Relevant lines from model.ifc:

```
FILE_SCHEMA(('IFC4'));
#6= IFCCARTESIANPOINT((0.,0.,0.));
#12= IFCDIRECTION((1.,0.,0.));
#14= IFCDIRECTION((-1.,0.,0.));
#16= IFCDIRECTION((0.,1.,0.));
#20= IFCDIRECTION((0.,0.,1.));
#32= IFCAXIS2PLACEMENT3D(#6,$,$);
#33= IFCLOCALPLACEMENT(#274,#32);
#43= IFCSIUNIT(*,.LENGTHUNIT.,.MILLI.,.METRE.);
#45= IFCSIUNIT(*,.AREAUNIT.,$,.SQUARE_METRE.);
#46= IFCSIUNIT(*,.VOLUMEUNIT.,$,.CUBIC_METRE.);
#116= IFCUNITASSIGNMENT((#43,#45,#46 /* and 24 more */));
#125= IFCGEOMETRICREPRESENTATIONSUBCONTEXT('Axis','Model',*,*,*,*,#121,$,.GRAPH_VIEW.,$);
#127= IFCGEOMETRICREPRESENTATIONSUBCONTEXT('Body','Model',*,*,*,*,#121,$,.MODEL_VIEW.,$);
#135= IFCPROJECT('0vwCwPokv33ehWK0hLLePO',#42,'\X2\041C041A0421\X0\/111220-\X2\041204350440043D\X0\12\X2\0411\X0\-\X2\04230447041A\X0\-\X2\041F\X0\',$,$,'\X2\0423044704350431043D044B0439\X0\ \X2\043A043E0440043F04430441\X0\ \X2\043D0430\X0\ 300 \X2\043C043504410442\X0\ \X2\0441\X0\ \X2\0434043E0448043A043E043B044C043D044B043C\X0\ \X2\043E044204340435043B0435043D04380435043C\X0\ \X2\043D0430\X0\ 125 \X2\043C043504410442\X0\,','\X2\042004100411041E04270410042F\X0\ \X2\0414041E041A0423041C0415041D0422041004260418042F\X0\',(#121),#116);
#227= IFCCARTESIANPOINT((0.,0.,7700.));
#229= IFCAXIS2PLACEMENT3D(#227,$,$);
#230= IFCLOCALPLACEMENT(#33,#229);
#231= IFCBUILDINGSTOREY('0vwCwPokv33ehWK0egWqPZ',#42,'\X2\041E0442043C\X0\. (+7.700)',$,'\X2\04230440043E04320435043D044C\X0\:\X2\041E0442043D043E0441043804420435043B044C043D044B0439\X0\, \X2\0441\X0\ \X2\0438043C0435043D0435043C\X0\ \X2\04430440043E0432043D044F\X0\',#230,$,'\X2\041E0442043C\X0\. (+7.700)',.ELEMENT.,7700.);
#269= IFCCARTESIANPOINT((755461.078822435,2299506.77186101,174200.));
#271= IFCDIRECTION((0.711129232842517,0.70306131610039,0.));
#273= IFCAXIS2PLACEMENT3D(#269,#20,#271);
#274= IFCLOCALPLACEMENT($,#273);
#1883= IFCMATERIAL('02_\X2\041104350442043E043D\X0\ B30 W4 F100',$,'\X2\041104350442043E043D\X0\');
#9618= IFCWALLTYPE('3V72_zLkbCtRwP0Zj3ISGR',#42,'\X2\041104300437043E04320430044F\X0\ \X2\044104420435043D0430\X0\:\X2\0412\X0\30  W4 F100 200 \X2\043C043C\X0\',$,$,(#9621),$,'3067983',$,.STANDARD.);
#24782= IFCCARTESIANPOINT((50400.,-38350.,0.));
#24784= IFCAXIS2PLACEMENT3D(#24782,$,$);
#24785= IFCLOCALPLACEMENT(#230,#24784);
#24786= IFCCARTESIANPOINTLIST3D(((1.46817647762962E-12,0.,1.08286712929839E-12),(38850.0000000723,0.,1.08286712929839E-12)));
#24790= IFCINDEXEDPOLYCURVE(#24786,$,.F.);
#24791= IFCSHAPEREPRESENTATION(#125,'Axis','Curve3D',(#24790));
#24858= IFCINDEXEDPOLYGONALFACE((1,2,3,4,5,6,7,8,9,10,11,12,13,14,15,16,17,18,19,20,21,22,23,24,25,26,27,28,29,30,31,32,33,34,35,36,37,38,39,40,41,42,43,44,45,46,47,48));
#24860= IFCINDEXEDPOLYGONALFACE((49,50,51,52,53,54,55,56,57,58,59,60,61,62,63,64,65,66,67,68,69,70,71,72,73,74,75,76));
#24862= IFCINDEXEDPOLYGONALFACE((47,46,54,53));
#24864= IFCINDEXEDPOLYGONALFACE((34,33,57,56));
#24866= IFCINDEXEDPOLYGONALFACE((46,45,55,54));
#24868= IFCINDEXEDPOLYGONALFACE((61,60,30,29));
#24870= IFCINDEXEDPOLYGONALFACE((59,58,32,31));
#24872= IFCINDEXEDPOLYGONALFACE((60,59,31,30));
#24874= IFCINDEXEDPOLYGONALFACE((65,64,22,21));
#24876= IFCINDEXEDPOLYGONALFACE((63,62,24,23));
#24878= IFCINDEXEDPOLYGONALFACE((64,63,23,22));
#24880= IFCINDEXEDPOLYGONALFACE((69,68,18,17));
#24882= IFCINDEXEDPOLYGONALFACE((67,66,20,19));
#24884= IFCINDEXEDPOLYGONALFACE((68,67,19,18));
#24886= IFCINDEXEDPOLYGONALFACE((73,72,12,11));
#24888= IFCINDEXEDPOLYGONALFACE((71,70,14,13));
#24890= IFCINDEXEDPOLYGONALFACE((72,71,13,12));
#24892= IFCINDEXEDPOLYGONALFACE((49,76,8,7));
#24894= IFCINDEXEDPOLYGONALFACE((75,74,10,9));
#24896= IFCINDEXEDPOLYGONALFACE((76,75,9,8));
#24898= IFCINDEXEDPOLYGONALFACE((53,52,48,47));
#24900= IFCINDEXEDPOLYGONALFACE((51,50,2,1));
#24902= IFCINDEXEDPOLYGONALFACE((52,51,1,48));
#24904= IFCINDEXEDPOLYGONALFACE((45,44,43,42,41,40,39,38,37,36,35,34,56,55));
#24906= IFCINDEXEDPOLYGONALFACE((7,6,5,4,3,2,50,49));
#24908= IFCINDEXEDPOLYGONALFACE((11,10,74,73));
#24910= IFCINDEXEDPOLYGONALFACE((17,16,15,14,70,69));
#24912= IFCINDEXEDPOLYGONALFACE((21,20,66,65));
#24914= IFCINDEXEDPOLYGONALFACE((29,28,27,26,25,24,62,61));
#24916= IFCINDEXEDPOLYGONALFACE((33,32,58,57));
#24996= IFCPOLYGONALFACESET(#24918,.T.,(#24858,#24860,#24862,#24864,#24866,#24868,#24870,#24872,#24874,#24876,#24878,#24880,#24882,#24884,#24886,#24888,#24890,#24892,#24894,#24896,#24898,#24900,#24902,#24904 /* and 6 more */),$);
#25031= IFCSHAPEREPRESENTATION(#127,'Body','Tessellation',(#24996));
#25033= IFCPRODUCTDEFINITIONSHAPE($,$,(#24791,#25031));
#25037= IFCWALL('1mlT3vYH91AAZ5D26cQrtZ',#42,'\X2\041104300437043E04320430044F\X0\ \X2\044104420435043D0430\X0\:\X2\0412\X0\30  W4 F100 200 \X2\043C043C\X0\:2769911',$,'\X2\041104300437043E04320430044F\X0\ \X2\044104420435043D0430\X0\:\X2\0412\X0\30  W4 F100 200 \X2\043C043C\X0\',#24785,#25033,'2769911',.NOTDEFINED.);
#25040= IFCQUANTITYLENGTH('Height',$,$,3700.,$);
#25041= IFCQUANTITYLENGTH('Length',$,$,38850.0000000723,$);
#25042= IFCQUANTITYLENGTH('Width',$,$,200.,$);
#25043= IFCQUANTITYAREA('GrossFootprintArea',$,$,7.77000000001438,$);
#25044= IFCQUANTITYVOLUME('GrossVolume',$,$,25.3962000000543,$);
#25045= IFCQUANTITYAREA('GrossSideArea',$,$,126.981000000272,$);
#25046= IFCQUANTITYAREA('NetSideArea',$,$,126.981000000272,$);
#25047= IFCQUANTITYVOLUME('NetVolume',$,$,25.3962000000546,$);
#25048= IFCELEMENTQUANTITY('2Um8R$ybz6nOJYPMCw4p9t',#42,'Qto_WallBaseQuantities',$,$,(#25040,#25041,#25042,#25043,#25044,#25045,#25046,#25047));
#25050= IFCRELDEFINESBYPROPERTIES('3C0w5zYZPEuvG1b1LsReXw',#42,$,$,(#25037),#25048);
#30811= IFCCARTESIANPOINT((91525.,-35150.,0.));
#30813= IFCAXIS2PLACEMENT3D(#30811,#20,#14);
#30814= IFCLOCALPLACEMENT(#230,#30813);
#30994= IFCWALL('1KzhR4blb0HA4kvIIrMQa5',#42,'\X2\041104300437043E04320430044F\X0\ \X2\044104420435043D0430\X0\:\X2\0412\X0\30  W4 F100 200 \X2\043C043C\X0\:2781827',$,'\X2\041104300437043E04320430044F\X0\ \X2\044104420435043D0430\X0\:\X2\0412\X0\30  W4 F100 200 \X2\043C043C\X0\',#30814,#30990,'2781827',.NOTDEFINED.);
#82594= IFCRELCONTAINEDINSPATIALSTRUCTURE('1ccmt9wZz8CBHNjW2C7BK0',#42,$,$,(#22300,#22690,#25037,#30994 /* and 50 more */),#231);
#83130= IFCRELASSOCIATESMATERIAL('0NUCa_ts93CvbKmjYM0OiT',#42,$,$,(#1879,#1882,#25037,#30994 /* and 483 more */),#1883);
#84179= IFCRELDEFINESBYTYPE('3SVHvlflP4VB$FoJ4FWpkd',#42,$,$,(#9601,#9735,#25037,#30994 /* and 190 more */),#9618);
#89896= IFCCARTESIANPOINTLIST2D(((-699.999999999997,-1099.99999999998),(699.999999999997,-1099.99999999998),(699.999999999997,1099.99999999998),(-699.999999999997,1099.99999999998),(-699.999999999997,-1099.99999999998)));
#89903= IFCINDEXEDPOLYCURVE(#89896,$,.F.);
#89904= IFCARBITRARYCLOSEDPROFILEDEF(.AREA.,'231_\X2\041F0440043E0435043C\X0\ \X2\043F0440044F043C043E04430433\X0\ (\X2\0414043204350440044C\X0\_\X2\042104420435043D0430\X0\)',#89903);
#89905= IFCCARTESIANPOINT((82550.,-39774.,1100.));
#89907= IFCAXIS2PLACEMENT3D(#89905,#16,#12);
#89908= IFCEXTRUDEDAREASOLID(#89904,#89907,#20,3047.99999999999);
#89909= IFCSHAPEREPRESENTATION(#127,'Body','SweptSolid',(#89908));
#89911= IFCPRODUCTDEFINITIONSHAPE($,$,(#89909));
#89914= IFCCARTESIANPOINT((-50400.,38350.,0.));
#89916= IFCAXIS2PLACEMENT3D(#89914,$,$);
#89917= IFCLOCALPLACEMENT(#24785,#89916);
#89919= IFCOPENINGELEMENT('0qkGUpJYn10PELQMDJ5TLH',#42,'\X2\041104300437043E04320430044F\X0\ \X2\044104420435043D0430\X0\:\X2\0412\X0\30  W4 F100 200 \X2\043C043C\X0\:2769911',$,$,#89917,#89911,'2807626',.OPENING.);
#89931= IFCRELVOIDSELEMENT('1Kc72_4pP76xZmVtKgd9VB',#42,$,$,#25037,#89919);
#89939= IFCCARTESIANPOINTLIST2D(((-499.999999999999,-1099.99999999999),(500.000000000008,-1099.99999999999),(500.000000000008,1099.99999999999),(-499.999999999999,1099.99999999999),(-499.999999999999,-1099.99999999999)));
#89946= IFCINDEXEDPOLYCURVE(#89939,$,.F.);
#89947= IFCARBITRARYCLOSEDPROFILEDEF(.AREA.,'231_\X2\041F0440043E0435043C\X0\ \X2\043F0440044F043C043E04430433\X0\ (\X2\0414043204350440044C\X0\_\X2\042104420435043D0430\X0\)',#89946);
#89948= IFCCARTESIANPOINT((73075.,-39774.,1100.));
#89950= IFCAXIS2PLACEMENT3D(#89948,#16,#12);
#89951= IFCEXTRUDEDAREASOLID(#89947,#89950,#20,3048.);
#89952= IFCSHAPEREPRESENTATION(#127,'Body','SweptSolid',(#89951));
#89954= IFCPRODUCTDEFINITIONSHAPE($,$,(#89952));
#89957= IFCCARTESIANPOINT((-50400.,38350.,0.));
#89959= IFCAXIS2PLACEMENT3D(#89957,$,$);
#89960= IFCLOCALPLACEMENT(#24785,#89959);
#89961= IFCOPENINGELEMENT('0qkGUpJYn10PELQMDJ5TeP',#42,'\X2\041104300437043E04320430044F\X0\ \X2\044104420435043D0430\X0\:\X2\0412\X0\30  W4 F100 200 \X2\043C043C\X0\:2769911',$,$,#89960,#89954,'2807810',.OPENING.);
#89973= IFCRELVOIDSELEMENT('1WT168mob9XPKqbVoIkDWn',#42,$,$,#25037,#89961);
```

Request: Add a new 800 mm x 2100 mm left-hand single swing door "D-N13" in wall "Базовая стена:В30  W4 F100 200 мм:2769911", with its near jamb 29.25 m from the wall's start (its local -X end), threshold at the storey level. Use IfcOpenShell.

```python
import numpy as np
import ifcopenshell
import ifcopenshell.api.feature
import ifcopenshell.api.geometry
import ifcopenshell.api.pset
import ifcopenshell.api.root
import ifcopenshell.api.spatial
import ifcopenshell.geom
import ifcopenshell.util.element
import ifcopenshell.util.placement
import ifcopenshell.util.representation
import ifcopenshell.util.shape
import ifcopenshell.util.unit

model = ifcopenshell.open("model.ifc")
unit_scale = ifcopenshell.util.unit.calculate_unit_scale(model)
area_scale = ifcopenshell.util.unit.calculate_unit_scale(model, "AREAUNIT")
volume_scale = ifcopenshell.util.unit.calculate_unit_scale(model, "VOLUMEUNIT")
settings = ifcopenshell.geom.settings()


def volume(element):
    """Net volume in cubic metres, openings subtracted."""
    shape = ifcopenshell.geom.create_shape(settings, element)
    return ifcopenshell.util.shape.get_volume(shape.geometry)


wall = model.by_guid("1mlT3vYH91AAZ5D26cQrtZ")
storey = ifcopenshell.util.element.get_container(wall, ifc_class="IfcBuildingStorey")
context = ifcopenshell.util.representation.get_context(model, "Model", "Body", "MODEL_VIEW")
before = volume(wall)

width, height, from_end, sill = 0.8, 2.1, 29.25, 0.0  # metres

# The wall runs along its own X axis, and the end named is its -X end.
wall_shape = ifcopenshell.geom.create_shape(settings, wall)
x, y, z = ifcopenshell.util.shape.get_vertices(wall_shape.geometry).T
start = x.min() + from_end
face, thickness = float(y.min()), float(y.max() - y.min())
wall_matrix = ifcopenshell.util.placement.get_local_placement(wall.ObjectPlacement)
level = ifcopenshell.util.placement.get_local_placement(storey.ObjectPlacement)[2, 3]


def in_wall(x, y):
    """Placement at x, y metres in the wall's axes, at sill height."""
    matrix = wall_matrix.copy()
    matrix[:, 3] = wall_matrix @ np.array([x / unit_scale, y / unit_scale, 0.0, 1.0])
    matrix[2, 3] = level + sill / unit_scale
    return matrix


# Opening: a box that overshoots both wall faces by 50 mm.
opening = ifcopenshell.api.root.create_entity(model, ifc_class="IfcOpeningElement", predefined_type="OPENING")
box = ifcopenshell.api.geometry.add_wall_representation(
    model, context=context, length=width, height=height, thickness=thickness + 0.1
)
ifcopenshell.api.geometry.assign_representation(model, product=opening, representation=box)
ifcopenshell.api.geometry.edit_object_placement(model, product=opening, matrix=in_wall(start, face - 0.05), is_si=False)
ifcopenshell.api.feature.add_feature(model, feature=opening, element=wall)

door = ifcopenshell.api.root.create_entity(model, ifc_class="IfcDoor", name="D-N13", predefined_type="DOOR")
door.OverallWidth, door.OverallHeight = width / unit_scale, height / unit_scale
door.OperationType = "SINGLE_SWING_LEFT"
body = ifcopenshell.api.geometry.add_door_representation(
    model,
    context=context,
    overall_width=door.OverallWidth,
    overall_height=door.OverallHeight,
    operation_type="SINGLE_SWING_LEFT",
    lining_properties={"LiningDepth": thickness / unit_scale, "ThresholdDepth": thickness / unit_scale},
)
ifcopenshell.api.geometry.assign_representation(model, product=door, representation=body)
ifcopenshell.api.spatial.assign_container(model, products=[door], relating_structure=storey)
ifcopenshell.api.feature.add_filling(model, opening=opening, element=door)

# The lining spans the wall, so the door starts at the wall face.
ifcopenshell.api.geometry.edit_object_placement(model, product=door, matrix=in_wall(start, face), is_si=False)

after = volume(wall)

# Update the wall's stored quantities.
qto = model.by_id(ifcopenshell.util.element.get_pset(wall, "Qto_WallBaseQuantities", should_inherit=False)["id"])
ifcopenshell.api.pset.edit_qto(model, qto=qto, properties={
    "NetSideArea": after / thickness / area_scale,
    "NetVolume": after / volume_scale,
})

print(f"wall volume {before:.3f} -> {after:.3f} m3")

model.write("model_updated.ifc")
```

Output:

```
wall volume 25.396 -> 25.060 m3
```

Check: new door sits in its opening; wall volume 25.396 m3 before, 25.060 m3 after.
